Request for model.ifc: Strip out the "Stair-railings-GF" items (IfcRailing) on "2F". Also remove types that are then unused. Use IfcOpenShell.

First a look at what the model holds.

```python
import ifcopenshell
import ifcopenshell.util.element

model = ifcopenshell.open("model.ifc")
print(model.schema)
storey = next(s for s in model.by_type("IfcBuildingStorey") if s.Name == "2F")
railings = [e for e in ifcopenshell.util.element.get_decomposition(storey) if e.is_a("IfcRailing")]
seen = {}
for e in railings:
    element_type = ifcopenshell.util.element.get_type(e)
    name = element_type.Name if element_type not in (None, e) else None
    seen[name] = seen.get(name, 0) + 1
for name, count in sorted(seen.items(), key=str):
    print(count, "x", name)
```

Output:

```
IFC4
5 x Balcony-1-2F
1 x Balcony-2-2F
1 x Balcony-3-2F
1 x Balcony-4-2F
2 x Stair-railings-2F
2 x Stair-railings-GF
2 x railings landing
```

```python
import ifcopenshell
import ifcopenshell.api.root
import ifcopenshell.util.element

model = ifcopenshell.open("model.ifc")

storey = next(s for s in model.by_type("IfcBuildingStorey") if s.Name == "2F")
railings = [e for e in ifcopenshell.util.element.get_decomposition(storey) if e.is_a("IfcRailing")]
targets = [e for e in railings if (t := ifcopenshell.util.element.get_type(e)) not in (None, e) and t.Name == "Stair-railings-GF"]
types = {ifcopenshell.util.element.get_type(e) for e in targets} - {None, *targets}

for e in targets:
    ifcopenshell.api.root.remove_product(model, product=e)
print(len(targets), "removed")

unused = [t for t in types if not ifcopenshell.util.element.get_types(t)]
for t in unused:
    ifcopenshell.api.root.remove_product(model, product=t)
print(len(unused), "unused types removed")

model.write("model_rev.ifc")
```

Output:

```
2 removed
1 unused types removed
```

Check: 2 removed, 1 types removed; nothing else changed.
